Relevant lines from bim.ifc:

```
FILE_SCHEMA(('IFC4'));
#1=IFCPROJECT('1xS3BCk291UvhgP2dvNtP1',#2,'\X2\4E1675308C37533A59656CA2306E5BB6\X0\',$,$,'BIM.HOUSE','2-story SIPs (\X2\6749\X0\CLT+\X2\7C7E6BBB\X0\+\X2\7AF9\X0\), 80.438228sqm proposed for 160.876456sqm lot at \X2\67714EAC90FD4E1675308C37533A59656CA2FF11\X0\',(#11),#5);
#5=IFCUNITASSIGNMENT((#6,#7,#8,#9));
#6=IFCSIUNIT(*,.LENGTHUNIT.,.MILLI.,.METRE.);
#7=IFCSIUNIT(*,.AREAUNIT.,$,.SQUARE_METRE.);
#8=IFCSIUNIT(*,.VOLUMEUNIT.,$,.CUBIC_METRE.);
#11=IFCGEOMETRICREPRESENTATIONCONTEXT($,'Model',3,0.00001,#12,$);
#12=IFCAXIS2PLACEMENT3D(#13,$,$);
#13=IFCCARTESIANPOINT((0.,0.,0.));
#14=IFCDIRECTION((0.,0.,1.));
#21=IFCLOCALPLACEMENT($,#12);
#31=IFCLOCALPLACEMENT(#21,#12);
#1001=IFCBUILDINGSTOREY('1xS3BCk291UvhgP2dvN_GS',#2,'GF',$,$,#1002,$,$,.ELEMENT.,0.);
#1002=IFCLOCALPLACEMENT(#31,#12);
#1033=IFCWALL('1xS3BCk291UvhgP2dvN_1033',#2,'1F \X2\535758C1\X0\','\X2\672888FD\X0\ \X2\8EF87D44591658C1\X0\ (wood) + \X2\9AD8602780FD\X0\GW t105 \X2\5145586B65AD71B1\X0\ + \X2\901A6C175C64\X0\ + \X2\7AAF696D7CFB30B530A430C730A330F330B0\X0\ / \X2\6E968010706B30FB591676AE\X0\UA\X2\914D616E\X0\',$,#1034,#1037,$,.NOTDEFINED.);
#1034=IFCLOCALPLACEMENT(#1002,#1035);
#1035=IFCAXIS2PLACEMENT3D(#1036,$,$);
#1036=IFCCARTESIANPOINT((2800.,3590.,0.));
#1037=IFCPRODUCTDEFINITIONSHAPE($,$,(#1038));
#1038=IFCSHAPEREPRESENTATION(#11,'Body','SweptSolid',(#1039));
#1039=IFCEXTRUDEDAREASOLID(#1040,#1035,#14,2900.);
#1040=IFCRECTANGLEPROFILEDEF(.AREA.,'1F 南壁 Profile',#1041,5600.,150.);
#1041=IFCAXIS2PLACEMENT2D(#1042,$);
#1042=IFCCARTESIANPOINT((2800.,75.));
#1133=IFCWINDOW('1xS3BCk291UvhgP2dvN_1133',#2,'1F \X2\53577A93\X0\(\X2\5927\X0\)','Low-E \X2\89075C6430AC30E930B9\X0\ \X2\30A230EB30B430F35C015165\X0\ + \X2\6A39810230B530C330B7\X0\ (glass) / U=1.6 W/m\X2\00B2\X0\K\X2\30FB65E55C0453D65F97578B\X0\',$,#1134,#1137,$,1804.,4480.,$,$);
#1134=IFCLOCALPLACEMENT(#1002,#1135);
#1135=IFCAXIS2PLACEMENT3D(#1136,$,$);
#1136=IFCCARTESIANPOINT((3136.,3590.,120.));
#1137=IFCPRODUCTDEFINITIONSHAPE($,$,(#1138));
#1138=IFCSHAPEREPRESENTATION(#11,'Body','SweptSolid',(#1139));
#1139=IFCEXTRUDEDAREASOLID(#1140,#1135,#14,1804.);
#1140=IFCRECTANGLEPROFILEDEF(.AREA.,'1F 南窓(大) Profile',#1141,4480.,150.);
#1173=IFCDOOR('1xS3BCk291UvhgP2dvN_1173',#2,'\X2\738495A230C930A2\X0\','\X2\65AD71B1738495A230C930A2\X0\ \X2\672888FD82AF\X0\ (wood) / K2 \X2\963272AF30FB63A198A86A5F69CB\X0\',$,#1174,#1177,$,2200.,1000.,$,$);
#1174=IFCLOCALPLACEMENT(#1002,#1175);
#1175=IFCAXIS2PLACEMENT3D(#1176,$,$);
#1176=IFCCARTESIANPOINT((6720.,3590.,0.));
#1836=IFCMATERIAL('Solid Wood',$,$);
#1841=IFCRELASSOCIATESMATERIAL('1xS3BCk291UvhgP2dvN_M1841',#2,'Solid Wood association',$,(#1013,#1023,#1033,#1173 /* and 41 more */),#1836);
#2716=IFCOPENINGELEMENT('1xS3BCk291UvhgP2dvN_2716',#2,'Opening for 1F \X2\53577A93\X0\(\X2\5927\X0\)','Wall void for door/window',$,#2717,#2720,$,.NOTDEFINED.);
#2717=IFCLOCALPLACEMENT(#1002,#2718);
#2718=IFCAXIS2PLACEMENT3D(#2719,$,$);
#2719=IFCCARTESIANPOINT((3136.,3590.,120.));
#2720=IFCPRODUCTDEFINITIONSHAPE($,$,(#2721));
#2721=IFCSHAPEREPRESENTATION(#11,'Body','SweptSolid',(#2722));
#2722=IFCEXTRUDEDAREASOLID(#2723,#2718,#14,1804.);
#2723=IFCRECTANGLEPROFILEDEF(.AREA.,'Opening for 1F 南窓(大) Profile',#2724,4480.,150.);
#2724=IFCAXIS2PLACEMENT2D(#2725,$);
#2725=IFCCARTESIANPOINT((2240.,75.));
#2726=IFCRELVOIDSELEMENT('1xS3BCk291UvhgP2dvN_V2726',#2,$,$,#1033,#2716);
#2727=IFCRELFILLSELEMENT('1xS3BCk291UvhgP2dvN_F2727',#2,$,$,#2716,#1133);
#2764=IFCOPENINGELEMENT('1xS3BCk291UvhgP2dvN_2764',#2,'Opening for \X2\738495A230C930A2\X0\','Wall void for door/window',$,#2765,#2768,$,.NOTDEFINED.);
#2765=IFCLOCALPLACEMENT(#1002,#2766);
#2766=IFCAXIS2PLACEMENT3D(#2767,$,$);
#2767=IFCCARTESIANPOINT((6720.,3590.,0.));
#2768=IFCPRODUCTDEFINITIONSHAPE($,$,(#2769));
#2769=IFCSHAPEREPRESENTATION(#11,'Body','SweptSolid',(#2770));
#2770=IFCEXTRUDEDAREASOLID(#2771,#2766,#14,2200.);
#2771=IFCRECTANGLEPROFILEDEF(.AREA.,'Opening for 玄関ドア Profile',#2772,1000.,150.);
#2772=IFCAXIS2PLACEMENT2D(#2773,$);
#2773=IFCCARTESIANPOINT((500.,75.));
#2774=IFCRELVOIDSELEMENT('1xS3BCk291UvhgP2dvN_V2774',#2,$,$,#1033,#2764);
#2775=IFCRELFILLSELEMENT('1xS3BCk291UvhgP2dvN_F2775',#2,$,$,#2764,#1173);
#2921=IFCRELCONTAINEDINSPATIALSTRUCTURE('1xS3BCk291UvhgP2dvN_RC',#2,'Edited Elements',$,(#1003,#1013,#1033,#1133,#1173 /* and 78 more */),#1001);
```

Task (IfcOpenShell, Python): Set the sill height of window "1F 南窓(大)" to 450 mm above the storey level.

```python
import numpy as np
import ifcopenshell
import ifcopenshell.api.geometry
import ifcopenshell.geom
import ifcopenshell.util.element
import ifcopenshell.util.placement
import ifcopenshell.util.shape
import ifcopenshell.util.unit

model = ifcopenshell.open("bim.ifc")
unit_scale = ifcopenshell.util.unit.calculate_unit_scale(model)

window = model.by_guid("1xS3BCk291UvhgP2dvN_1133")
opening = window.FillsVoids[0].RelatingOpeningElement
storey = ifcopenshell.util.element.get_container(window, ifc_class="IfcBuildingStorey")
level = ifcopenshell.util.placement.get_local_placement(storey.ObjectPlacement)[2, 3]

# The opening's origin need not be at the sill, so measure its lowest point.
shape = ifcopenshell.geom.create_shape(ifcopenshell.geom.settings(), opening)
bottom = ifcopenshell.util.shape.get_shape_bottom_elevation(shape, shape.geometry) / unit_scale
dz = level + 450.0 - bottom

shift = np.array([0.0, 0.0, dz])
# The window is not placed relative to its opening, so move both.
for product in (opening, window):
    matrix = ifcopenshell.util.placement.get_local_placement(product.ObjectPlacement)
    matrix[:3, 3] += shift
    ifcopenshell.api.geometry.edit_object_placement(model, product=product, matrix=matrix, is_si=False)

print(f"moved by {dz * unit_scale:+.3f} m")

model.write("bim_rev.ifc")
```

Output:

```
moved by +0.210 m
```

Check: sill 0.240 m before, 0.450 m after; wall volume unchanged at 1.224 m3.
